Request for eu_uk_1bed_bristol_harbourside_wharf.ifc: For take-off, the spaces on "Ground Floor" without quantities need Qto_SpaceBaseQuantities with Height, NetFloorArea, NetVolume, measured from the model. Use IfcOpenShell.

First a look at what the model holds.

```python
import ifcopenshell
import ifcopenshell.util.element
import ifcopenshell.util.unit

model = ifcopenshell.open("eu_uk_1bed_bristol_harbourside_wharf.ifc")
print(model.schema)
for unit_type in ("LENGTHUNIT", "AREAUNIT", "VOLUMEUNIT"):
    print(unit_type, ifcopenshell.util.unit.calculate_unit_scale(model, unit_type))
storey = next(s for s in model.by_type("IfcBuildingStorey") if s.Name == "Ground Floor")
spaces = [e for e in ifcopenshell.util.element.get_decomposition(storey) if e.is_a("IfcSpace")]
for e in sorted(spaces, key=lambda e: e.id()):
    print(e.id(), e.is_a(), e.Name, list(ifcopenshell.util.element.get_psets(e, qtos_only=True)), sep=" | ")
```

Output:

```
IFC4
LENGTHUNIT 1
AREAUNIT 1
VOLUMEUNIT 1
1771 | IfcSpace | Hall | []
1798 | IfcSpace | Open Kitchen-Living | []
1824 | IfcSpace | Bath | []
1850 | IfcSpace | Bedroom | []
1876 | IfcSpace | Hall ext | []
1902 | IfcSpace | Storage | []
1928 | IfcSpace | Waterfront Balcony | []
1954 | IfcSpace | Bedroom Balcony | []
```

```python
import ifcopenshell
import ifcopenshell.api.pset
import ifcopenshell.geom
import ifcopenshell.util.element
import ifcopenshell.util.shape
import ifcopenshell.util.unit

model = ifcopenshell.open("eu_uk_1bed_bristol_harbourside_wharf.ifc")
unit_scale = ifcopenshell.util.unit.calculate_unit_scale(model)
area_scale = ifcopenshell.util.unit.calculate_unit_scale(model, "AREAUNIT")
volume_scale = ifcopenshell.util.unit.calculate_unit_scale(model, "VOLUMEUNIT")
settings = ifcopenshell.geom.settings()

storey = next(s for s in model.by_type("IfcBuildingStorey") if s.Name == "Ground Floor")
spaces = [e for e in ifcopenshell.util.element.get_decomposition(storey) if e.is_a("IfcSpace")]

for e in sorted(spaces, key=lambda e: e.id()):
    if ifcopenshell.util.element.get_psets(e, qtos_only=True, should_inherit=False):
        continue
    # Geometry comes back in metres, in the element's own axes.
    shape = ifcopenshell.geom.create_shape(settings, e)
    values = {
        "Height": ifcopenshell.util.shape.get_z(shape.geometry) / unit_scale,
        "NetFloorArea": ifcopenshell.util.shape.get_footprint_area(shape.geometry) / area_scale,
        "NetVolume": ifcopenshell.util.shape.get_volume(shape.geometry) / volume_scale,
    }
    qto = ifcopenshell.api.pset.add_qto(model, product=e, name="Qto_SpaceBaseQuantities")
    ifcopenshell.api.pset.edit_qto(model, qto=qto, properties=values)
    print(e.id(), {k: round(v, 3) for k, v in values.items()})

model.write("eu_uk_1bed_bristol_harbourside_wharf_v2.ifc")
```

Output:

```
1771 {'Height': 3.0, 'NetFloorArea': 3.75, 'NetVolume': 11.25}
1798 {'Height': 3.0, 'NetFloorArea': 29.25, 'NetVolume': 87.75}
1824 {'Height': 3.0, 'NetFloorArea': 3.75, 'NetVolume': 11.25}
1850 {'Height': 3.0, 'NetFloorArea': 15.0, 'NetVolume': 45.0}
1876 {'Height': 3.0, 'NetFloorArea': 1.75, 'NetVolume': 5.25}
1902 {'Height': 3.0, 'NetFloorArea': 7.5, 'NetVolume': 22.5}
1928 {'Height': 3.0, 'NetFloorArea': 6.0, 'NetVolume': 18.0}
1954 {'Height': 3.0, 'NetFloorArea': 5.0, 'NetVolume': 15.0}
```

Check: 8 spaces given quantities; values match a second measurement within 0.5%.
